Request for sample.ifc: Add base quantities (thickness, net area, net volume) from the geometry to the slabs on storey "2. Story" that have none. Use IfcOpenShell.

First a look at what the model holds.

```python
import ifcopenshell
import ifcopenshell.util.element
import ifcopenshell.util.unit

model = ifcopenshell.open("sample.ifc")
print(model.schema)
for unit_type in ("LENGTHUNIT", "AREAUNIT", "VOLUMEUNIT"):
    print(unit_type, ifcopenshell.util.unit.calculate_unit_scale(model, unit_type))
storey = next(s for s in model.by_type("IfcBuildingStorey") if s.Name == "2. Story")
slabs = [e for e in ifcopenshell.util.element.get_decomposition(storey) if e.is_a("IfcSlab")]
for e in sorted(slabs, key=lambda e: e.id()):
    print(e.id(), e.is_a(), e.Name, list(ifcopenshell.util.element.get_psets(e, qtos_only=True)), sep=" | ")
```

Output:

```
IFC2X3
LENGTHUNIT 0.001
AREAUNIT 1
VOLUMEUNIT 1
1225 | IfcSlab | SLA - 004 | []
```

```python
import ifcopenshell
import ifcopenshell.api.pset
import ifcopenshell.geom
import ifcopenshell.util.element
import ifcopenshell.util.shape
import ifcopenshell.util.unit

model = ifcopenshell.open("sample.ifc")
unit_scale = ifcopenshell.util.unit.calculate_unit_scale(model)
area_scale = ifcopenshell.util.unit.calculate_unit_scale(model, "AREAUNIT")
volume_scale = ifcopenshell.util.unit.calculate_unit_scale(model, "VOLUMEUNIT")
settings = ifcopenshell.geom.settings()

storey = next(s for s in model.by_type("IfcBuildingStorey") if s.Name == "2. Story")
slabs = [e for e in ifcopenshell.util.element.get_decomposition(storey) if e.is_a("IfcSlab")]

for e in sorted(slabs, key=lambda e: e.id()):
    if ifcopenshell.util.element.get_psets(e, qtos_only=True, should_inherit=False):
        continue
    # Geometry comes back in metres, in the element's own axes.
    shape = ifcopenshell.geom.create_shape(settings, e)
    values = {
        "Width": ifcopenshell.util.shape.get_z(shape.geometry) / unit_scale,
        "NetArea": ifcopenshell.util.shape.get_footprint_area(shape.geometry) / area_scale,
        "NetVolume": ifcopenshell.util.shape.get_volume(shape.geometry) / volume_scale,
    }
    qto = ifcopenshell.api.pset.add_qto(model, product=e, name="BaseQuantities")
    ifcopenshell.api.pset.edit_qto(model, qto=qto, properties=values)
    print(e.id(), {k: round(v, 3) for k, v in values.items()})

model.write("sample-out.ifc")
```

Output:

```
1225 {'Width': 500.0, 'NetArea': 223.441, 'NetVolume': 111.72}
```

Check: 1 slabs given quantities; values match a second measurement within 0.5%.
